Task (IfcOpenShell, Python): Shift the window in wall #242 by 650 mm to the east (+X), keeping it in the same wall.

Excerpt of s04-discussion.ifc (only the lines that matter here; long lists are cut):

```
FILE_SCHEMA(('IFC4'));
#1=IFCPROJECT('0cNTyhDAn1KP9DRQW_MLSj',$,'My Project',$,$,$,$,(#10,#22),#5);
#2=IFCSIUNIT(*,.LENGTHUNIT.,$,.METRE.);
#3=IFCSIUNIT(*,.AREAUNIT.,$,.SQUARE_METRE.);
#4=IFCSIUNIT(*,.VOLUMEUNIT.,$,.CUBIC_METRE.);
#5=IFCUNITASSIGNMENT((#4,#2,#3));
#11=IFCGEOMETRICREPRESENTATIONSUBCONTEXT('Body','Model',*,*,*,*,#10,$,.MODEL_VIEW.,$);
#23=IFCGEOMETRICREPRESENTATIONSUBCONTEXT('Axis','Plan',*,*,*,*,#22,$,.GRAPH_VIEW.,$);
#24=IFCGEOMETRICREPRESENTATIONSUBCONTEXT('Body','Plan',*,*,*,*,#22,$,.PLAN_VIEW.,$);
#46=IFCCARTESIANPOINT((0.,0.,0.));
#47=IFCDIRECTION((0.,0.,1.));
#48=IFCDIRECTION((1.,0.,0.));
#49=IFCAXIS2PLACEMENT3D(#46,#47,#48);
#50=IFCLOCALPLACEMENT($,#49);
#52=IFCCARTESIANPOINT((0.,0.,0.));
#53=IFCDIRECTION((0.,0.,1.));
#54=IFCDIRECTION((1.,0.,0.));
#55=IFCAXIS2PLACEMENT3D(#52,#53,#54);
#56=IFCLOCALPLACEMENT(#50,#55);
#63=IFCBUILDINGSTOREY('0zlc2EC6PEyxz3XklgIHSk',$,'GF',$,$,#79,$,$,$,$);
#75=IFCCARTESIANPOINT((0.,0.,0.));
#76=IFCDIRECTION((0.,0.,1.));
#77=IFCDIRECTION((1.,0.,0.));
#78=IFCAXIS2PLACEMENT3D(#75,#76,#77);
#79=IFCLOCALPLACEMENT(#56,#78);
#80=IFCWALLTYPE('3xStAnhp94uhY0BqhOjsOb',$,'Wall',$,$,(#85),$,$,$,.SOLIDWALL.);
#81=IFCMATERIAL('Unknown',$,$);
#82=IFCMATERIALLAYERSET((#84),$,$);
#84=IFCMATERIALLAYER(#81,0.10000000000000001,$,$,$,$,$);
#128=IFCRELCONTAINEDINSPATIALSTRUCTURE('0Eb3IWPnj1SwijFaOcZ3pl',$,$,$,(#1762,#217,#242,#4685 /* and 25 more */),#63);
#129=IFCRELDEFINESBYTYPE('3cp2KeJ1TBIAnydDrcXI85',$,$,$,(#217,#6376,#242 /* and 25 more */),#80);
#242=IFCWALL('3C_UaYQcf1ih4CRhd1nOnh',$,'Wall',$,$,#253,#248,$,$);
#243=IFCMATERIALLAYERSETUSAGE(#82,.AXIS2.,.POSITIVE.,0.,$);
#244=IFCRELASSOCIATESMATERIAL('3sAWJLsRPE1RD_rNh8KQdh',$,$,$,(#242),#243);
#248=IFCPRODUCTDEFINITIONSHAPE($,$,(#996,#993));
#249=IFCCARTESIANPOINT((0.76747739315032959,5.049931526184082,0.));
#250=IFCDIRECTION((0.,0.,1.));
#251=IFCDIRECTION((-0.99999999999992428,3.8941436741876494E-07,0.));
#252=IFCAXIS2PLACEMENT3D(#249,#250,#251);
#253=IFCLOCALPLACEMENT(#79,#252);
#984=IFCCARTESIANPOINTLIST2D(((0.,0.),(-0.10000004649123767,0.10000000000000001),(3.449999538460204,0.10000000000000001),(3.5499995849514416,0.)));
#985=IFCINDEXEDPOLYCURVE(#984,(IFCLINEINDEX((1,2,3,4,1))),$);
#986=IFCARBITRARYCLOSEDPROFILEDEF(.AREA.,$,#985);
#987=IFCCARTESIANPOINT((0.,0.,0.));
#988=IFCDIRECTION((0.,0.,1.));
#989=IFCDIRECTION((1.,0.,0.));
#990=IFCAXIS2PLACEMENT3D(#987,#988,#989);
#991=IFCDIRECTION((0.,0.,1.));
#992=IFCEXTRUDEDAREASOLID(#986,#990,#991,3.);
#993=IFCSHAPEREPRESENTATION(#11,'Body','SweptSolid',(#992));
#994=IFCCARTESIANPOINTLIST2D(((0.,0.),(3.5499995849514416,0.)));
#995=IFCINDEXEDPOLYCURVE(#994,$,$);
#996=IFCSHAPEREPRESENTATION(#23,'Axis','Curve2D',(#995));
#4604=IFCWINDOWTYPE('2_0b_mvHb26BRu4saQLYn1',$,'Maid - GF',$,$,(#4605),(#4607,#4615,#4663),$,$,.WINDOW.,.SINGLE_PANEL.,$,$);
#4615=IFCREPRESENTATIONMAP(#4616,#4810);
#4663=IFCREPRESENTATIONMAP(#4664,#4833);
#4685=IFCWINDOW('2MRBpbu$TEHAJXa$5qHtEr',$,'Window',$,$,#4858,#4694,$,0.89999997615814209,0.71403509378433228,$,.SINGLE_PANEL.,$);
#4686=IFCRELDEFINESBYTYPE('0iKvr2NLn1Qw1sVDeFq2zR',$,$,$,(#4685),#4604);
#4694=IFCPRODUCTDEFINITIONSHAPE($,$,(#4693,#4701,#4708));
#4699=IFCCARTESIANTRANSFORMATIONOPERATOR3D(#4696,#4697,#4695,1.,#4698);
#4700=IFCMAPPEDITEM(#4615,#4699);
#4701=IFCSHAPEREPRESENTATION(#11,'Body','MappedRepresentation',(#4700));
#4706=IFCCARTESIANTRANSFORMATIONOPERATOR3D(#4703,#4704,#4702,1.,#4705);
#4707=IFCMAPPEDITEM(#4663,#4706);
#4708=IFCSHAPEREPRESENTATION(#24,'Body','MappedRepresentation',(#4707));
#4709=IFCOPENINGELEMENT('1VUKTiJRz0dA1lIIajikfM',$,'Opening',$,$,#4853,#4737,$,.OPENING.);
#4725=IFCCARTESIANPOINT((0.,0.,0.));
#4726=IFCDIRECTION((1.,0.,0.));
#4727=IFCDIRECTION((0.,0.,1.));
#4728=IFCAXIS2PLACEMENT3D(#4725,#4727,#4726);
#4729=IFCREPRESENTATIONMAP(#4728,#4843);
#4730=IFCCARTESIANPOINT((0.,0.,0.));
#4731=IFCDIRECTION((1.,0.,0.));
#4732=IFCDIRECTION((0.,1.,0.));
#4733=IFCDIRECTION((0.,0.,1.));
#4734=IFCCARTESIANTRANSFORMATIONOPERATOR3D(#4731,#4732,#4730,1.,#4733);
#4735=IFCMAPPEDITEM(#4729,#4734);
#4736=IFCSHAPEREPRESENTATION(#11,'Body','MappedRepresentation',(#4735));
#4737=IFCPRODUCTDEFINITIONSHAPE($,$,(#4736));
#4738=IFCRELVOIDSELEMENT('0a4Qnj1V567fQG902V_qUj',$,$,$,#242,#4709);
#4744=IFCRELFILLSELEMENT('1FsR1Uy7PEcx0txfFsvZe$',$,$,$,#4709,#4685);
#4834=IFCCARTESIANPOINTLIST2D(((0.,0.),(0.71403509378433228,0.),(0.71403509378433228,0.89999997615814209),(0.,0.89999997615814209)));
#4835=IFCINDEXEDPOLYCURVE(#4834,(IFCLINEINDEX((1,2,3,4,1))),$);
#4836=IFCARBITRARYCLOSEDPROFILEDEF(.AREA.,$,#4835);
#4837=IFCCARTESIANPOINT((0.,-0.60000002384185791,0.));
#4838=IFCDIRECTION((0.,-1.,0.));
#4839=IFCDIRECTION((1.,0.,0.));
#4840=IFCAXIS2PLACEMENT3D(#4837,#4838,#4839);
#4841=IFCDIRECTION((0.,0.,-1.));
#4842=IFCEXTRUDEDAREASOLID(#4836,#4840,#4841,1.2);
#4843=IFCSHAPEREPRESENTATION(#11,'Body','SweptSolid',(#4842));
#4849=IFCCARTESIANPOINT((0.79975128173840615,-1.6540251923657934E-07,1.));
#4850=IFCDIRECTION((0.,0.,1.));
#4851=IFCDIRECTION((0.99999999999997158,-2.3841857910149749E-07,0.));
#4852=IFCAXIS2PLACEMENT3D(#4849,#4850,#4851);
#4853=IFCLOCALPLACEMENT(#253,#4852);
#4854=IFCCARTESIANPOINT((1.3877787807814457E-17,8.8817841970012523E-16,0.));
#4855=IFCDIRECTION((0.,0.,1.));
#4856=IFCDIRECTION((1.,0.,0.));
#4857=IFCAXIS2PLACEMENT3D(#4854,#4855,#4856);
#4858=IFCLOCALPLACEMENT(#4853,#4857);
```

```python
import ifcopenshell
import ifcopenshell.api.geometry
import ifcopenshell.util.placement
import ifcopenshell.util.unit

model = ifcopenshell.open("s04-discussion.ifc")
unit_scale = ifcopenshell.util.unit.calculate_unit_scale(model)

window = model.by_id(4685)
opening = window.FillsVoids[0].RelatingOpeningElement
wall = opening.VoidsElements[0].RelatingBuildingElement

wall_matrix = ifcopenshell.util.placement.get_local_placement(wall.ObjectPlacement)
shift = wall_matrix[:3, 0] * -0.65 / unit_scale
before = ifcopenshell.util.placement.get_local_placement(window.ObjectPlacement)[:3, 3].copy()

# The window is placed relative to its opening, so it follows when the opening moves.
matrix = ifcopenshell.util.placement.get_local_placement(opening.ObjectPlacement)
matrix[:3, 3] += shift
ifcopenshell.api.geometry.edit_object_placement(
    model, product=opening, matrix=matrix, is_si=False, should_transform_children=True
)

after = ifcopenshell.util.placement.get_local_placement(window.ObjectPlacement)[:3, 3]
print("window moved by", (after - before).round(3) + 0.0)

model.write("s04-discussion_rev.ifc")
```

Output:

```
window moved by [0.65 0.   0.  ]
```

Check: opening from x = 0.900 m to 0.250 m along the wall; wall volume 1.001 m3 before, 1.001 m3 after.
